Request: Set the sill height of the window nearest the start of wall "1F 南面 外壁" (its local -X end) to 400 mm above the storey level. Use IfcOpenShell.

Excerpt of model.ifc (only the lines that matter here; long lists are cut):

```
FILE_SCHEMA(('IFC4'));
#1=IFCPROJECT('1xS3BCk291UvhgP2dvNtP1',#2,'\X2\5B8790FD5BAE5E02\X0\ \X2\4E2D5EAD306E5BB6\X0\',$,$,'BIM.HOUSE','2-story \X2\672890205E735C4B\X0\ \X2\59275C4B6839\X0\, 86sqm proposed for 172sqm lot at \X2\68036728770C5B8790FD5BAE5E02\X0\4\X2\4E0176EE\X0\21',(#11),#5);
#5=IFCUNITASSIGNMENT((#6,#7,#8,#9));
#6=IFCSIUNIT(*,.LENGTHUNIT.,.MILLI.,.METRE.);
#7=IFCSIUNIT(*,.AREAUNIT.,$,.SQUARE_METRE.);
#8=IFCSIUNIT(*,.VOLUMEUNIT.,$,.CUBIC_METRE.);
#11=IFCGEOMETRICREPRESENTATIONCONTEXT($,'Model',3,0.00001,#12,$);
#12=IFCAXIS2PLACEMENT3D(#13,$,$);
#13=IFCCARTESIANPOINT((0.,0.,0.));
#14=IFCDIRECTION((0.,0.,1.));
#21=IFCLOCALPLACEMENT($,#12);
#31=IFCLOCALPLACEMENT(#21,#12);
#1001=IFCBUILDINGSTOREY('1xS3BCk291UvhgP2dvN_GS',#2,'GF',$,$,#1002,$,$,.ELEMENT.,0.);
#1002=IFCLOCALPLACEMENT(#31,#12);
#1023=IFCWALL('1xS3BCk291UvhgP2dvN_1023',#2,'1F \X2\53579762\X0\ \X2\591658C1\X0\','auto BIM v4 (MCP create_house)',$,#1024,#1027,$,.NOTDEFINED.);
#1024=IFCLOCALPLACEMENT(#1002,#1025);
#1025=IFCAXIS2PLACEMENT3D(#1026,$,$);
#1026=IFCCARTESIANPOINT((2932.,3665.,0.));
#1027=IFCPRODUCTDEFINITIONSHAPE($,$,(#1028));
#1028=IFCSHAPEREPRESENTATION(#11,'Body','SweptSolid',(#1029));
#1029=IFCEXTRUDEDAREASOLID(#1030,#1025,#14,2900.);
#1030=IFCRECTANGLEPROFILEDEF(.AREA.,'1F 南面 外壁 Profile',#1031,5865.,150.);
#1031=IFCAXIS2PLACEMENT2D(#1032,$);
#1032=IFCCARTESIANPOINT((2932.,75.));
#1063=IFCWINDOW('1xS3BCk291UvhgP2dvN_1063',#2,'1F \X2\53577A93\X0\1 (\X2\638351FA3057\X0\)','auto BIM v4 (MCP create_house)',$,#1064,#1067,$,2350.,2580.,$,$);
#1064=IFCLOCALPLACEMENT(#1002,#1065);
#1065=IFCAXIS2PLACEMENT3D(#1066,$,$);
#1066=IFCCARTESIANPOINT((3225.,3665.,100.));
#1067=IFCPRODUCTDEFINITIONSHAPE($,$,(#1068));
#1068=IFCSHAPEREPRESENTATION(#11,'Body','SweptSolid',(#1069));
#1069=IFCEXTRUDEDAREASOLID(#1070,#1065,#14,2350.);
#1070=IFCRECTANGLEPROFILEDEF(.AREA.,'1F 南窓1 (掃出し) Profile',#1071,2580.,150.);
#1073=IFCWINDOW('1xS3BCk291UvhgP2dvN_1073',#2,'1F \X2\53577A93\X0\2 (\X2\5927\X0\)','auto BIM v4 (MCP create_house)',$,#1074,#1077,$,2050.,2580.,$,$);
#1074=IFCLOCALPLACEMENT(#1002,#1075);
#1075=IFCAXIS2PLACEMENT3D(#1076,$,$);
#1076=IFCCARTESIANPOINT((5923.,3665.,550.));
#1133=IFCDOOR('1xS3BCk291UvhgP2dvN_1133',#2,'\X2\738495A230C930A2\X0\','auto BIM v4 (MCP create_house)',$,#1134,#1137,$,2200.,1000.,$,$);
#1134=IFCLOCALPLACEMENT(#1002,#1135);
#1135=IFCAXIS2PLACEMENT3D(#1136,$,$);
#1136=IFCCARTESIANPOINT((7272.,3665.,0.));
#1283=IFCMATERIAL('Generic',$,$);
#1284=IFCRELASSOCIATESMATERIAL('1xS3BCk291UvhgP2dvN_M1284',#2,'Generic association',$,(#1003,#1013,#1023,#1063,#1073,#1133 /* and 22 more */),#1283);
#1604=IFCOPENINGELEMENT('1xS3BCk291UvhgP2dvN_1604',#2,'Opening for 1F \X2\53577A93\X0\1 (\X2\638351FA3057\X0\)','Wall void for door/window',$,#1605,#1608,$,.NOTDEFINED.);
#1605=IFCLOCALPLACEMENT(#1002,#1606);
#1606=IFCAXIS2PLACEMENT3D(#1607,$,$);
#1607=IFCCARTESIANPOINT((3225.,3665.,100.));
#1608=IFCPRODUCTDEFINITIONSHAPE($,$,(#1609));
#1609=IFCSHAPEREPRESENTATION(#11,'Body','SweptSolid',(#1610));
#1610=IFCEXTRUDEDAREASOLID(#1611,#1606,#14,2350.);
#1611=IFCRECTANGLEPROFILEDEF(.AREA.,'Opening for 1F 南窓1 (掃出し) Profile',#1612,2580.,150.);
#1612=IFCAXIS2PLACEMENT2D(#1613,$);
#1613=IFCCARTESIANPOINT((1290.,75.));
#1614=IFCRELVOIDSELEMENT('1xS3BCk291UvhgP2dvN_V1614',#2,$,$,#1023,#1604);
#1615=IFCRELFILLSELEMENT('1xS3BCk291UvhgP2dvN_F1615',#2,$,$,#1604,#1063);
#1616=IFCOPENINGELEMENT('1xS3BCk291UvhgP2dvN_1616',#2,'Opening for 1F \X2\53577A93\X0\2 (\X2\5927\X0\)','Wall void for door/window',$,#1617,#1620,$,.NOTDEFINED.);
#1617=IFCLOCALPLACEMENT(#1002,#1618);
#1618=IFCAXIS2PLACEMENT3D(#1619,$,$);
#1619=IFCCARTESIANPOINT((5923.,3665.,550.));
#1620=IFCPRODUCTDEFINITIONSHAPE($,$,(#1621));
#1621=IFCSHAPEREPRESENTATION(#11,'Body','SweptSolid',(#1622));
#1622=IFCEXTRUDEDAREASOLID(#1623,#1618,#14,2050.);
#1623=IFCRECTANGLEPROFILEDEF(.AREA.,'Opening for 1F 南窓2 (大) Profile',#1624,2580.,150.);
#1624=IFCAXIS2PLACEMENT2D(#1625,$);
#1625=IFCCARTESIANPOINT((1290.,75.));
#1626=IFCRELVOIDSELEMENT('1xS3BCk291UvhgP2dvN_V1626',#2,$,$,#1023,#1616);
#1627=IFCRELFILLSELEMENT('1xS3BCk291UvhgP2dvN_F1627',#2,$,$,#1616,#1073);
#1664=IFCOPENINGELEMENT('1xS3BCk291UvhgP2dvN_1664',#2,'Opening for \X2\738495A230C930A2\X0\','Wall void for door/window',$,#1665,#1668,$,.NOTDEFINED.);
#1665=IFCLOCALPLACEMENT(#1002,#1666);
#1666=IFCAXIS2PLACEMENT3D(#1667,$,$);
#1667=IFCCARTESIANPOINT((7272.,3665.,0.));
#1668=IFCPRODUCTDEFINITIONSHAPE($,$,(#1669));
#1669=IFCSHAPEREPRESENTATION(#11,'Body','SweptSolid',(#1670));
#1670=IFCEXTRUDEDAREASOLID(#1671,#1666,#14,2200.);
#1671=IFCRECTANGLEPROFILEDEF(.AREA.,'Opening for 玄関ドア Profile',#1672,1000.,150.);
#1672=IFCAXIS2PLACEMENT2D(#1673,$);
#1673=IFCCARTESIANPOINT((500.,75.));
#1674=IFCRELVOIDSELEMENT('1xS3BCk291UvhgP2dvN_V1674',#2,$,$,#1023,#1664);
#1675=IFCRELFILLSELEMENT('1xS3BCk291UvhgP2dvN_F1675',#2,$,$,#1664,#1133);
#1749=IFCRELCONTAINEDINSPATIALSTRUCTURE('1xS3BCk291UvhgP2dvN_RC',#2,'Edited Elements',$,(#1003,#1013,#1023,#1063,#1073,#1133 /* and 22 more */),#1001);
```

```python
import numpy as np
import ifcopenshell
import ifcopenshell.api.geometry
import ifcopenshell.geom
import ifcopenshell.util.element
import ifcopenshell.util.placement
import ifcopenshell.util.shape
import ifcopenshell.util.unit

model = ifcopenshell.open("model.ifc")
unit_scale = ifcopenshell.util.unit.calculate_unit_scale(model)

window = model.by_guid("1xS3BCk291UvhgP2dvN_1063")
opening = window.FillsVoids[0].RelatingOpeningElement
storey = ifcopenshell.util.element.get_container(window, ifc_class="IfcBuildingStorey")
level = ifcopenshell.util.placement.get_local_placement(storey.ObjectPlacement)[2, 3]

# The opening's origin need not be at the sill, so measure its lowest point.
shape = ifcopenshell.geom.create_shape(ifcopenshell.geom.settings(), opening)
bottom = ifcopenshell.util.shape.get_shape_bottom_elevation(shape, shape.geometry) / unit_scale
dz = level + 400.0 - bottom

shift = np.array([0.0, 0.0, dz])
# The window is not placed relative to its opening, so move both.
for product in (opening, window):
    matrix = ifcopenshell.util.placement.get_local_placement(product.ObjectPlacement)
    matrix[:3, 3] += shift
    ifcopenshell.api.geometry.edit_object_placement(model, product=product, matrix=matrix, is_si=False)

print(f"moved by {dz * unit_scale:+.3f} m")

model.write("model_rev.ifc")
```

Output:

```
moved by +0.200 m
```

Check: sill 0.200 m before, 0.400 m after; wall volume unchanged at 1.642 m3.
